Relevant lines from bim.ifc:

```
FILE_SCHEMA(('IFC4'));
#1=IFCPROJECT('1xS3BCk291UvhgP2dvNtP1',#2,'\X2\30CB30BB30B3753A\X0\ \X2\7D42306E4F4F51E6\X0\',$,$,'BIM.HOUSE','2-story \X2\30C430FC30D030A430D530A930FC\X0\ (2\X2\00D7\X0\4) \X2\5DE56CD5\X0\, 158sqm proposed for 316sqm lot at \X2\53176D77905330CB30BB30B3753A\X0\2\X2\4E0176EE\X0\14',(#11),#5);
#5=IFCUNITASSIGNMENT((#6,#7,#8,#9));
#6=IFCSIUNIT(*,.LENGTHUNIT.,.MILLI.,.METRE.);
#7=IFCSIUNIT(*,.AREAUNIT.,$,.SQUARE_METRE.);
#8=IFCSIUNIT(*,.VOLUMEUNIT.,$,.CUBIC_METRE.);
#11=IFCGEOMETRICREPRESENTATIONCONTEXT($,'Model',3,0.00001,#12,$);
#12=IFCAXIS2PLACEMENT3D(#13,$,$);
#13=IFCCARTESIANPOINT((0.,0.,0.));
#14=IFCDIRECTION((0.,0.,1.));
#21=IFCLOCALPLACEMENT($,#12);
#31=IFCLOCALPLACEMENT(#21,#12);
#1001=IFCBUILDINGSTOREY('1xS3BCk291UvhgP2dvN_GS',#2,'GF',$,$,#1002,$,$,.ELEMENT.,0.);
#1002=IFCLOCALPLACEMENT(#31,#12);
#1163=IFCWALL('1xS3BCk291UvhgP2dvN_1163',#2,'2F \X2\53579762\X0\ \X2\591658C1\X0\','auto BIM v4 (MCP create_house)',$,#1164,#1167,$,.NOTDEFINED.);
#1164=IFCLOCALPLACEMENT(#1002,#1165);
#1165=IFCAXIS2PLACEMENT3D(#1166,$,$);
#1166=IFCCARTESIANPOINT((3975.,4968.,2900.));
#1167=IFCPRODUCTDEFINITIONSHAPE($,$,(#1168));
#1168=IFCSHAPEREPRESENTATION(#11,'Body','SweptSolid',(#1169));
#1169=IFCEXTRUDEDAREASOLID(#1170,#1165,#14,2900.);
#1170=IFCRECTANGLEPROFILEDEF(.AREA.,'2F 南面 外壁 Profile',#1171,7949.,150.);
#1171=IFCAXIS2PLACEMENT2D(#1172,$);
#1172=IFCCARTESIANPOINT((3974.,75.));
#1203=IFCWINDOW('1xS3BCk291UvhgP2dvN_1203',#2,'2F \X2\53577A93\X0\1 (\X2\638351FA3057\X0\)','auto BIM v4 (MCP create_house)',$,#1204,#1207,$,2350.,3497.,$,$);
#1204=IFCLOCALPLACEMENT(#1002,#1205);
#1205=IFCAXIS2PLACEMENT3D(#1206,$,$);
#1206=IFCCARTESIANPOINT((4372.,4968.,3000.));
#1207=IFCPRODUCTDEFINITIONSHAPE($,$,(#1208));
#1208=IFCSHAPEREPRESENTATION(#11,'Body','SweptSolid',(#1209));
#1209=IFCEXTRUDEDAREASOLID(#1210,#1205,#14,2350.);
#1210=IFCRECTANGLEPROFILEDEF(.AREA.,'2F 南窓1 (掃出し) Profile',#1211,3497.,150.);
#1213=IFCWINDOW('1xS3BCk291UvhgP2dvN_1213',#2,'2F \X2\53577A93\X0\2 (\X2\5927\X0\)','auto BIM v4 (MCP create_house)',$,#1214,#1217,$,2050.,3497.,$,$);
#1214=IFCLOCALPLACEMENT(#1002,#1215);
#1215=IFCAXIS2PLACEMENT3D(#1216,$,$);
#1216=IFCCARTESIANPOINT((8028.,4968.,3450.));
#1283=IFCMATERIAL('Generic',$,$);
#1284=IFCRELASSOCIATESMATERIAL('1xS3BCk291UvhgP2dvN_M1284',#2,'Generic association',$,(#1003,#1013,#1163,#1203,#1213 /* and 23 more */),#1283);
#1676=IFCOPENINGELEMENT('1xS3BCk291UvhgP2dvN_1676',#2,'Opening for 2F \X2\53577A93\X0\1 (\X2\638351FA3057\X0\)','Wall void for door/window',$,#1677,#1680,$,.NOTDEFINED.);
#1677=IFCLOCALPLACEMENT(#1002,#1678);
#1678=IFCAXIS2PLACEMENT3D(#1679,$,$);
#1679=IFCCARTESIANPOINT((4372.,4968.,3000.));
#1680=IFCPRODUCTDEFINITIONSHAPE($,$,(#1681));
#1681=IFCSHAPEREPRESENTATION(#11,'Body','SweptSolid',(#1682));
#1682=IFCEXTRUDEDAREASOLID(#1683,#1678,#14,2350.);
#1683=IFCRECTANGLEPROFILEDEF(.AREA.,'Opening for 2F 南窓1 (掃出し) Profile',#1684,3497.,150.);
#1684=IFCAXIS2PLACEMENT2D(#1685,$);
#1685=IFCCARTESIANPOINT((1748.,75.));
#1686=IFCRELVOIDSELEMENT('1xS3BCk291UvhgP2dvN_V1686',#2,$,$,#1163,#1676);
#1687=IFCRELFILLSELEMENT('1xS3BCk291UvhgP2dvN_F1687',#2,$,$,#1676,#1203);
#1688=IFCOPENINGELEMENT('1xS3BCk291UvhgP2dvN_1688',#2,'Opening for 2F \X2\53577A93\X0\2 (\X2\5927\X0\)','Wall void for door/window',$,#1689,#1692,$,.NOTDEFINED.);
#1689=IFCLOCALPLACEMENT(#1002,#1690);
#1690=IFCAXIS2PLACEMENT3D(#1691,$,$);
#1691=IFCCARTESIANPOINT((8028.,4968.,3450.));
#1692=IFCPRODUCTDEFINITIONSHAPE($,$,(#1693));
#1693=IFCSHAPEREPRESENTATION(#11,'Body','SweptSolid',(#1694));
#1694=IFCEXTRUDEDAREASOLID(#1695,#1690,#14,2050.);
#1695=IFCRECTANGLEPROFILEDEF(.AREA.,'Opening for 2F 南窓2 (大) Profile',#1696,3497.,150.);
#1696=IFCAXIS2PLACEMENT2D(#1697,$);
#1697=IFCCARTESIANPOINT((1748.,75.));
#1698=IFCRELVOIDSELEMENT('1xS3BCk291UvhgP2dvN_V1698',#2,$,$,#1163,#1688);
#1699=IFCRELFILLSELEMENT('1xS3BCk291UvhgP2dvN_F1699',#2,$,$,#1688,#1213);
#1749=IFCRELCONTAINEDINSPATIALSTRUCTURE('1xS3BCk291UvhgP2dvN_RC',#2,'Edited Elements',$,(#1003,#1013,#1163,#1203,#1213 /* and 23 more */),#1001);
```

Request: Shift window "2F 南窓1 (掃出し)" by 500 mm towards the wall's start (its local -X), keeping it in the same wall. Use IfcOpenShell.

```python
import ifcopenshell
import ifcopenshell.api.geometry
import ifcopenshell.util.placement
import ifcopenshell.util.unit

model = ifcopenshell.open("bim.ifc")
unit_scale = ifcopenshell.util.unit.calculate_unit_scale(model)

window = model.by_id(1203)
opening = window.FillsVoids[0].RelatingOpeningElement
wall = opening.VoidsElements[0].RelatingBuildingElement

wall_matrix = ifcopenshell.util.placement.get_local_placement(wall.ObjectPlacement)
shift = wall_matrix[:3, 0] * -0.5 / unit_scale
before = ifcopenshell.util.placement.get_local_placement(window.ObjectPlacement)[:3, 3].copy()

# The window is not placed relative to its opening, so move both.
for product in (opening, window):
    matrix = ifcopenshell.util.placement.get_local_placement(product.ObjectPlacement)
    matrix[:3, 3] += shift
    ifcopenshell.api.geometry.edit_object_placement(model, product=product, matrix=matrix, is_si=False)

after = ifcopenshell.util.placement.get_local_placement(window.ObjectPlacement)[:3, 3]
print("window moved by", (after - before).round(3) + 0.0)

model.write("bim_v2.ifc")
```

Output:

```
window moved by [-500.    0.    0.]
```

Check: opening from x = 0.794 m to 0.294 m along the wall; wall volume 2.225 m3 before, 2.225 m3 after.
